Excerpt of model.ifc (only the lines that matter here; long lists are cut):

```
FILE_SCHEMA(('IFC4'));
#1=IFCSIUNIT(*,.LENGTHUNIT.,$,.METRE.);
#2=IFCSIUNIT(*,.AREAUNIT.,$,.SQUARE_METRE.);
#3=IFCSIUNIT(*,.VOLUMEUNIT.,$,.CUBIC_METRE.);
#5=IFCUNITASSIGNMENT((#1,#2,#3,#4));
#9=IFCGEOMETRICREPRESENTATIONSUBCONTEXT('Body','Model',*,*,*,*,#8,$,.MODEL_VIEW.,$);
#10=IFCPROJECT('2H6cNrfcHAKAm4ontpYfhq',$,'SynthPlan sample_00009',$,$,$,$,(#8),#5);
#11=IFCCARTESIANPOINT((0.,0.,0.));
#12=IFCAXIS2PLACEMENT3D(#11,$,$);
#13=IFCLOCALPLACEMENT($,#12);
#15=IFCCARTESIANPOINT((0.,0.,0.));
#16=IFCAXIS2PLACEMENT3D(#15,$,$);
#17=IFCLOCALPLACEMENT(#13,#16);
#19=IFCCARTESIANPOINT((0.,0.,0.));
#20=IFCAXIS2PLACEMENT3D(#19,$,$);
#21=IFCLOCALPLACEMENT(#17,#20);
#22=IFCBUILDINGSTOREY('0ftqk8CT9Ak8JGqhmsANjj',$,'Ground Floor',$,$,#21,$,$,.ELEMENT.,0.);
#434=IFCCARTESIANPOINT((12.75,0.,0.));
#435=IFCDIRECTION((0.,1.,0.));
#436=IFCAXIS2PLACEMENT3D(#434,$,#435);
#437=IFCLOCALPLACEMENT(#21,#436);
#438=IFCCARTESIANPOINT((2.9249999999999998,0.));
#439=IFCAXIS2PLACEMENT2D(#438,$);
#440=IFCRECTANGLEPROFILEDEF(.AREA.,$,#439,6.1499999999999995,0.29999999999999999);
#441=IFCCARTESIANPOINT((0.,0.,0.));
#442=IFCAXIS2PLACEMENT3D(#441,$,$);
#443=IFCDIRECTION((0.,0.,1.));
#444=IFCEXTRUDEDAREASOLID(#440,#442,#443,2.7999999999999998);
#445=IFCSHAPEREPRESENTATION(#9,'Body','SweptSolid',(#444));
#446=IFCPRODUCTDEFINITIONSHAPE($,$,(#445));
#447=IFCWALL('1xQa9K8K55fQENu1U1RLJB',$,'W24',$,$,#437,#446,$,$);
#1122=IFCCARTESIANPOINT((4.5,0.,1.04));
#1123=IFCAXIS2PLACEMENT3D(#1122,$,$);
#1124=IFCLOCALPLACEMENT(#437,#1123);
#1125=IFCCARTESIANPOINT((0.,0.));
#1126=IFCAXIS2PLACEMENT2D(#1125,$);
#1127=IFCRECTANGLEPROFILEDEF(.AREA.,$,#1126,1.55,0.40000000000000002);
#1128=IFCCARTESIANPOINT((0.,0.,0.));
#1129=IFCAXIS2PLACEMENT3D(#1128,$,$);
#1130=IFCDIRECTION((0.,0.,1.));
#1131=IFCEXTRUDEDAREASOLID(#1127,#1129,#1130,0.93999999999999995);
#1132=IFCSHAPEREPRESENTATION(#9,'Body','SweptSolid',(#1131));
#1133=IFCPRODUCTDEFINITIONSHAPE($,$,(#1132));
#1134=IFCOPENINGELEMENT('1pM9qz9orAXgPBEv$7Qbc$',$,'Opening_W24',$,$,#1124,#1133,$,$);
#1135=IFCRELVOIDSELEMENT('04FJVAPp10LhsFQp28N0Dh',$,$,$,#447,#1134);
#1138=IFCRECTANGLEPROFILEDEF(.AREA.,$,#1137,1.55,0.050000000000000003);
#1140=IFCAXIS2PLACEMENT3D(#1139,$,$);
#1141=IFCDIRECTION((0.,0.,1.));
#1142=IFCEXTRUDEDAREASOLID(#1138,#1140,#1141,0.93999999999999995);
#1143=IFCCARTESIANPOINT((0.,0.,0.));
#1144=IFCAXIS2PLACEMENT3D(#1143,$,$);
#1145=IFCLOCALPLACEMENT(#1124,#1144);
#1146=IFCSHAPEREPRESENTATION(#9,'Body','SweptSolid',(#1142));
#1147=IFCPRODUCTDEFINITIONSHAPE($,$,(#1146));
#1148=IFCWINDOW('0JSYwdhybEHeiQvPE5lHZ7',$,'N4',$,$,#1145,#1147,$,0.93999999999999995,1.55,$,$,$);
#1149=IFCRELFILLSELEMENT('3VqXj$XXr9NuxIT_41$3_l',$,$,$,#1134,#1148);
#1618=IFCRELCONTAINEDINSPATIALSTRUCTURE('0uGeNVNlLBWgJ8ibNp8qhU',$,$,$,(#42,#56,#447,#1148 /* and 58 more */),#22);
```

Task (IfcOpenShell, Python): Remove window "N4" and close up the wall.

```python
import ifcopenshell
import ifcopenshell.api.feature
import ifcopenshell.api.root
import ifcopenshell.geom
import ifcopenshell.util.shape

model = ifcopenshell.open("model.ifc")
settings = ifcopenshell.geom.settings()


def volume(element):
    """Net volume in cubic metres, openings subtracted."""
    shape = ifcopenshell.geom.create_shape(settings, element)
    return ifcopenshell.util.shape.get_volume(shape.geometry)


window = model.by_id(1148)
opening = window.FillsVoids[0].RelatingOpeningElement
wall = opening.VoidsElements[0].RelatingBuildingElement
before = volume(wall)

ifcopenshell.api.root.remove_product(model, product=window)
ifcopenshell.api.feature.remove_feature(model, feature=opening)

after = volume(wall)

print(f"wall volume {before:.3f} -> {after:.3f} m3")

model.write("model_updated.ifc")
```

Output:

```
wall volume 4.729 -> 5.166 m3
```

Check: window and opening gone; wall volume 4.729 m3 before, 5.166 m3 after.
